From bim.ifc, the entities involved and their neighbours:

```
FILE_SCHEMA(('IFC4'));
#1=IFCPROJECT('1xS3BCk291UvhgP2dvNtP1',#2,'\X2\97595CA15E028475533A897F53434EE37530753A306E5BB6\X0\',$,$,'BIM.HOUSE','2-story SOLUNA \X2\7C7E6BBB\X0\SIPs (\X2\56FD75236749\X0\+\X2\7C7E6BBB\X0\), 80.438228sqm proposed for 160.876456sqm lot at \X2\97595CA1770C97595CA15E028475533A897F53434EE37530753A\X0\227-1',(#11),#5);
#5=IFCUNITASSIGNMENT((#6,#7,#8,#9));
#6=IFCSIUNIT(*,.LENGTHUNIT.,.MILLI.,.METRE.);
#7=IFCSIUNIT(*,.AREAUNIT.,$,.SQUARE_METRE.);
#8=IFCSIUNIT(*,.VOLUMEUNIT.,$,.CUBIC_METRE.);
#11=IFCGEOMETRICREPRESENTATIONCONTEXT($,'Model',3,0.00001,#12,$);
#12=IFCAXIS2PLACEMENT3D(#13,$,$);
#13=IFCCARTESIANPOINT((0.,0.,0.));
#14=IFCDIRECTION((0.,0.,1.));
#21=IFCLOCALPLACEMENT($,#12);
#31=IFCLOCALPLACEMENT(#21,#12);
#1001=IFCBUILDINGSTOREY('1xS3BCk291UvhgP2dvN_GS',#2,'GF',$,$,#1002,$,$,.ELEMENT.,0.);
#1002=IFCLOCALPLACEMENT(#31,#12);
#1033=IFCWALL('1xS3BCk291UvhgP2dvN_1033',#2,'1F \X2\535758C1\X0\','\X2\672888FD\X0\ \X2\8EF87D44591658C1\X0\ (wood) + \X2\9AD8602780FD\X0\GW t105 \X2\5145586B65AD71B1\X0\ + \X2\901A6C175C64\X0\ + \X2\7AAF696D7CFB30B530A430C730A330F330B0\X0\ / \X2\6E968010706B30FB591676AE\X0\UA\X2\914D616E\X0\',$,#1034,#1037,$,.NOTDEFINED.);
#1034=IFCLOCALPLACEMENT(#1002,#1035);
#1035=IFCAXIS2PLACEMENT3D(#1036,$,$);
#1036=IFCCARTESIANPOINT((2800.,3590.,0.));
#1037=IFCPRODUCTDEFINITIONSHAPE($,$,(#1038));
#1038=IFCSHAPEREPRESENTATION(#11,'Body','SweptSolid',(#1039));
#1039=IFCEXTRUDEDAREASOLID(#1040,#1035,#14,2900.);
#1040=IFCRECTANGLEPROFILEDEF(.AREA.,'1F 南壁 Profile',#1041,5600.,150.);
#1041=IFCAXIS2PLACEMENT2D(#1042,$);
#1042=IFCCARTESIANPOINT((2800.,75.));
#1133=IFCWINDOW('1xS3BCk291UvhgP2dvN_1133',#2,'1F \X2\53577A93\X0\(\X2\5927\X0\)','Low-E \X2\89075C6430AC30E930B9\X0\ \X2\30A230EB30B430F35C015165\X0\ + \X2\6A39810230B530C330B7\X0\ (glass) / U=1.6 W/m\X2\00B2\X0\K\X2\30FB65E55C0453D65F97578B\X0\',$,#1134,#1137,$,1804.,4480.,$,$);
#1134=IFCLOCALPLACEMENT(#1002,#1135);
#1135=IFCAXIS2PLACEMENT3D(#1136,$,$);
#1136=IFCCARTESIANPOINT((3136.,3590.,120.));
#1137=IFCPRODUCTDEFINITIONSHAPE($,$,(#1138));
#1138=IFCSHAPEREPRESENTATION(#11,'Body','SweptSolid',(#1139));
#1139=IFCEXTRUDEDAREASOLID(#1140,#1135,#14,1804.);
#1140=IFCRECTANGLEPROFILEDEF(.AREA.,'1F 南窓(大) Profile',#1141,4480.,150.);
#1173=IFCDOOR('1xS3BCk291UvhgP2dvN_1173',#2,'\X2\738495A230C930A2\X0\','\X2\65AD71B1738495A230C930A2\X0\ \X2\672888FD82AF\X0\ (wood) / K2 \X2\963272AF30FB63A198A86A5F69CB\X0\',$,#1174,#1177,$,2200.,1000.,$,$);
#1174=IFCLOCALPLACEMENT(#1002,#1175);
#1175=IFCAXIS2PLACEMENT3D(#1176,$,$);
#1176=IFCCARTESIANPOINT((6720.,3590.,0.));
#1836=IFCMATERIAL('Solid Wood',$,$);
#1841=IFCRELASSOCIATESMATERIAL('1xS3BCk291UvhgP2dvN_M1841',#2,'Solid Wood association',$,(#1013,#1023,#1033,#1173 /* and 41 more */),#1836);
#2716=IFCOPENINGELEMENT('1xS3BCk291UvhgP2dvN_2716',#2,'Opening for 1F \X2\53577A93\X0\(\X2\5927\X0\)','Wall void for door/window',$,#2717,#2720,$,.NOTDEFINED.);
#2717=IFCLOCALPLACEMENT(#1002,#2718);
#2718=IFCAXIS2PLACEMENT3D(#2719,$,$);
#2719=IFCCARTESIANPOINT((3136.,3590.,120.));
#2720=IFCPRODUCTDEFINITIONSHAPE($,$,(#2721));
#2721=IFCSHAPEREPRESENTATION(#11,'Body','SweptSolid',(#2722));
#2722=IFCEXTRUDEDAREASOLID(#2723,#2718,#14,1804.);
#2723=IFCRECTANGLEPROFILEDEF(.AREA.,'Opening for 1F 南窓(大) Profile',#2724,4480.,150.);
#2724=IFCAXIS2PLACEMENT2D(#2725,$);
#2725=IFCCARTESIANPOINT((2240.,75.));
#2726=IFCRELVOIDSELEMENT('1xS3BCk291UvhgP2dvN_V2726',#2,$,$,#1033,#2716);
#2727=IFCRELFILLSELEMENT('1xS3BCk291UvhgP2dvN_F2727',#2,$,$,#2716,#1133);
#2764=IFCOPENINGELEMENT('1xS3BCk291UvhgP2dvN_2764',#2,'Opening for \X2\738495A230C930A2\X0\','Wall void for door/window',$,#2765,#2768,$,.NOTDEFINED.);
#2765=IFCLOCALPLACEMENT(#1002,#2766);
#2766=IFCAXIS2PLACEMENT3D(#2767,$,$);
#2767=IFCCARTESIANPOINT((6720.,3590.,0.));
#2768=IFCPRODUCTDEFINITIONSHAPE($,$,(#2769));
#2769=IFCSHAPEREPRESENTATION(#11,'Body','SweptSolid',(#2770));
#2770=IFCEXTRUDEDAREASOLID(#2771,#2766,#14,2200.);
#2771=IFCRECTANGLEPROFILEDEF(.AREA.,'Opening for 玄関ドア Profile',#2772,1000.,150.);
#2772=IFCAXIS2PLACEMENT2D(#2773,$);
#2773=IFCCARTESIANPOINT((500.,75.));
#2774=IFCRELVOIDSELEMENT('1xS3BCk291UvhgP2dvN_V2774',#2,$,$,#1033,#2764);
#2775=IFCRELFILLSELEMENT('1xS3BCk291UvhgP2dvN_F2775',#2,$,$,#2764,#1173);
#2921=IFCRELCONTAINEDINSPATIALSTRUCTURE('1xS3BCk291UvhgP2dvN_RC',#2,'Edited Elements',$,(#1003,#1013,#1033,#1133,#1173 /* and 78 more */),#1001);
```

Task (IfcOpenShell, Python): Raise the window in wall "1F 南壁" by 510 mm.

```python
import numpy as np
import ifcopenshell
import ifcopenshell.api.geometry
import ifcopenshell.util.placement
import ifcopenshell.util.unit

model = ifcopenshell.open("bim.ifc")
unit_scale = ifcopenshell.util.unit.calculate_unit_scale(model)

window = model.by_guid("1xS3BCk291UvhgP2dvN_1133")
opening = window.FillsVoids[0].RelatingOpeningElement
dz = 0.51 / unit_scale

shift = np.array([0.0, 0.0, dz])
# The window is not placed relative to its opening, so move both.
for product in (opening, window):
    matrix = ifcopenshell.util.placement.get_local_placement(product.ObjectPlacement)
    matrix[:3, 3] += shift
    ifcopenshell.api.geometry.edit_object_placement(model, product=product, matrix=matrix, is_si=False)

print(f"moved by {dz * unit_scale:+.3f} m")

model.write("bim-out.ifc")
```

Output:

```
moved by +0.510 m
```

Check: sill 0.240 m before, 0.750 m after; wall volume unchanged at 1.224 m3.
